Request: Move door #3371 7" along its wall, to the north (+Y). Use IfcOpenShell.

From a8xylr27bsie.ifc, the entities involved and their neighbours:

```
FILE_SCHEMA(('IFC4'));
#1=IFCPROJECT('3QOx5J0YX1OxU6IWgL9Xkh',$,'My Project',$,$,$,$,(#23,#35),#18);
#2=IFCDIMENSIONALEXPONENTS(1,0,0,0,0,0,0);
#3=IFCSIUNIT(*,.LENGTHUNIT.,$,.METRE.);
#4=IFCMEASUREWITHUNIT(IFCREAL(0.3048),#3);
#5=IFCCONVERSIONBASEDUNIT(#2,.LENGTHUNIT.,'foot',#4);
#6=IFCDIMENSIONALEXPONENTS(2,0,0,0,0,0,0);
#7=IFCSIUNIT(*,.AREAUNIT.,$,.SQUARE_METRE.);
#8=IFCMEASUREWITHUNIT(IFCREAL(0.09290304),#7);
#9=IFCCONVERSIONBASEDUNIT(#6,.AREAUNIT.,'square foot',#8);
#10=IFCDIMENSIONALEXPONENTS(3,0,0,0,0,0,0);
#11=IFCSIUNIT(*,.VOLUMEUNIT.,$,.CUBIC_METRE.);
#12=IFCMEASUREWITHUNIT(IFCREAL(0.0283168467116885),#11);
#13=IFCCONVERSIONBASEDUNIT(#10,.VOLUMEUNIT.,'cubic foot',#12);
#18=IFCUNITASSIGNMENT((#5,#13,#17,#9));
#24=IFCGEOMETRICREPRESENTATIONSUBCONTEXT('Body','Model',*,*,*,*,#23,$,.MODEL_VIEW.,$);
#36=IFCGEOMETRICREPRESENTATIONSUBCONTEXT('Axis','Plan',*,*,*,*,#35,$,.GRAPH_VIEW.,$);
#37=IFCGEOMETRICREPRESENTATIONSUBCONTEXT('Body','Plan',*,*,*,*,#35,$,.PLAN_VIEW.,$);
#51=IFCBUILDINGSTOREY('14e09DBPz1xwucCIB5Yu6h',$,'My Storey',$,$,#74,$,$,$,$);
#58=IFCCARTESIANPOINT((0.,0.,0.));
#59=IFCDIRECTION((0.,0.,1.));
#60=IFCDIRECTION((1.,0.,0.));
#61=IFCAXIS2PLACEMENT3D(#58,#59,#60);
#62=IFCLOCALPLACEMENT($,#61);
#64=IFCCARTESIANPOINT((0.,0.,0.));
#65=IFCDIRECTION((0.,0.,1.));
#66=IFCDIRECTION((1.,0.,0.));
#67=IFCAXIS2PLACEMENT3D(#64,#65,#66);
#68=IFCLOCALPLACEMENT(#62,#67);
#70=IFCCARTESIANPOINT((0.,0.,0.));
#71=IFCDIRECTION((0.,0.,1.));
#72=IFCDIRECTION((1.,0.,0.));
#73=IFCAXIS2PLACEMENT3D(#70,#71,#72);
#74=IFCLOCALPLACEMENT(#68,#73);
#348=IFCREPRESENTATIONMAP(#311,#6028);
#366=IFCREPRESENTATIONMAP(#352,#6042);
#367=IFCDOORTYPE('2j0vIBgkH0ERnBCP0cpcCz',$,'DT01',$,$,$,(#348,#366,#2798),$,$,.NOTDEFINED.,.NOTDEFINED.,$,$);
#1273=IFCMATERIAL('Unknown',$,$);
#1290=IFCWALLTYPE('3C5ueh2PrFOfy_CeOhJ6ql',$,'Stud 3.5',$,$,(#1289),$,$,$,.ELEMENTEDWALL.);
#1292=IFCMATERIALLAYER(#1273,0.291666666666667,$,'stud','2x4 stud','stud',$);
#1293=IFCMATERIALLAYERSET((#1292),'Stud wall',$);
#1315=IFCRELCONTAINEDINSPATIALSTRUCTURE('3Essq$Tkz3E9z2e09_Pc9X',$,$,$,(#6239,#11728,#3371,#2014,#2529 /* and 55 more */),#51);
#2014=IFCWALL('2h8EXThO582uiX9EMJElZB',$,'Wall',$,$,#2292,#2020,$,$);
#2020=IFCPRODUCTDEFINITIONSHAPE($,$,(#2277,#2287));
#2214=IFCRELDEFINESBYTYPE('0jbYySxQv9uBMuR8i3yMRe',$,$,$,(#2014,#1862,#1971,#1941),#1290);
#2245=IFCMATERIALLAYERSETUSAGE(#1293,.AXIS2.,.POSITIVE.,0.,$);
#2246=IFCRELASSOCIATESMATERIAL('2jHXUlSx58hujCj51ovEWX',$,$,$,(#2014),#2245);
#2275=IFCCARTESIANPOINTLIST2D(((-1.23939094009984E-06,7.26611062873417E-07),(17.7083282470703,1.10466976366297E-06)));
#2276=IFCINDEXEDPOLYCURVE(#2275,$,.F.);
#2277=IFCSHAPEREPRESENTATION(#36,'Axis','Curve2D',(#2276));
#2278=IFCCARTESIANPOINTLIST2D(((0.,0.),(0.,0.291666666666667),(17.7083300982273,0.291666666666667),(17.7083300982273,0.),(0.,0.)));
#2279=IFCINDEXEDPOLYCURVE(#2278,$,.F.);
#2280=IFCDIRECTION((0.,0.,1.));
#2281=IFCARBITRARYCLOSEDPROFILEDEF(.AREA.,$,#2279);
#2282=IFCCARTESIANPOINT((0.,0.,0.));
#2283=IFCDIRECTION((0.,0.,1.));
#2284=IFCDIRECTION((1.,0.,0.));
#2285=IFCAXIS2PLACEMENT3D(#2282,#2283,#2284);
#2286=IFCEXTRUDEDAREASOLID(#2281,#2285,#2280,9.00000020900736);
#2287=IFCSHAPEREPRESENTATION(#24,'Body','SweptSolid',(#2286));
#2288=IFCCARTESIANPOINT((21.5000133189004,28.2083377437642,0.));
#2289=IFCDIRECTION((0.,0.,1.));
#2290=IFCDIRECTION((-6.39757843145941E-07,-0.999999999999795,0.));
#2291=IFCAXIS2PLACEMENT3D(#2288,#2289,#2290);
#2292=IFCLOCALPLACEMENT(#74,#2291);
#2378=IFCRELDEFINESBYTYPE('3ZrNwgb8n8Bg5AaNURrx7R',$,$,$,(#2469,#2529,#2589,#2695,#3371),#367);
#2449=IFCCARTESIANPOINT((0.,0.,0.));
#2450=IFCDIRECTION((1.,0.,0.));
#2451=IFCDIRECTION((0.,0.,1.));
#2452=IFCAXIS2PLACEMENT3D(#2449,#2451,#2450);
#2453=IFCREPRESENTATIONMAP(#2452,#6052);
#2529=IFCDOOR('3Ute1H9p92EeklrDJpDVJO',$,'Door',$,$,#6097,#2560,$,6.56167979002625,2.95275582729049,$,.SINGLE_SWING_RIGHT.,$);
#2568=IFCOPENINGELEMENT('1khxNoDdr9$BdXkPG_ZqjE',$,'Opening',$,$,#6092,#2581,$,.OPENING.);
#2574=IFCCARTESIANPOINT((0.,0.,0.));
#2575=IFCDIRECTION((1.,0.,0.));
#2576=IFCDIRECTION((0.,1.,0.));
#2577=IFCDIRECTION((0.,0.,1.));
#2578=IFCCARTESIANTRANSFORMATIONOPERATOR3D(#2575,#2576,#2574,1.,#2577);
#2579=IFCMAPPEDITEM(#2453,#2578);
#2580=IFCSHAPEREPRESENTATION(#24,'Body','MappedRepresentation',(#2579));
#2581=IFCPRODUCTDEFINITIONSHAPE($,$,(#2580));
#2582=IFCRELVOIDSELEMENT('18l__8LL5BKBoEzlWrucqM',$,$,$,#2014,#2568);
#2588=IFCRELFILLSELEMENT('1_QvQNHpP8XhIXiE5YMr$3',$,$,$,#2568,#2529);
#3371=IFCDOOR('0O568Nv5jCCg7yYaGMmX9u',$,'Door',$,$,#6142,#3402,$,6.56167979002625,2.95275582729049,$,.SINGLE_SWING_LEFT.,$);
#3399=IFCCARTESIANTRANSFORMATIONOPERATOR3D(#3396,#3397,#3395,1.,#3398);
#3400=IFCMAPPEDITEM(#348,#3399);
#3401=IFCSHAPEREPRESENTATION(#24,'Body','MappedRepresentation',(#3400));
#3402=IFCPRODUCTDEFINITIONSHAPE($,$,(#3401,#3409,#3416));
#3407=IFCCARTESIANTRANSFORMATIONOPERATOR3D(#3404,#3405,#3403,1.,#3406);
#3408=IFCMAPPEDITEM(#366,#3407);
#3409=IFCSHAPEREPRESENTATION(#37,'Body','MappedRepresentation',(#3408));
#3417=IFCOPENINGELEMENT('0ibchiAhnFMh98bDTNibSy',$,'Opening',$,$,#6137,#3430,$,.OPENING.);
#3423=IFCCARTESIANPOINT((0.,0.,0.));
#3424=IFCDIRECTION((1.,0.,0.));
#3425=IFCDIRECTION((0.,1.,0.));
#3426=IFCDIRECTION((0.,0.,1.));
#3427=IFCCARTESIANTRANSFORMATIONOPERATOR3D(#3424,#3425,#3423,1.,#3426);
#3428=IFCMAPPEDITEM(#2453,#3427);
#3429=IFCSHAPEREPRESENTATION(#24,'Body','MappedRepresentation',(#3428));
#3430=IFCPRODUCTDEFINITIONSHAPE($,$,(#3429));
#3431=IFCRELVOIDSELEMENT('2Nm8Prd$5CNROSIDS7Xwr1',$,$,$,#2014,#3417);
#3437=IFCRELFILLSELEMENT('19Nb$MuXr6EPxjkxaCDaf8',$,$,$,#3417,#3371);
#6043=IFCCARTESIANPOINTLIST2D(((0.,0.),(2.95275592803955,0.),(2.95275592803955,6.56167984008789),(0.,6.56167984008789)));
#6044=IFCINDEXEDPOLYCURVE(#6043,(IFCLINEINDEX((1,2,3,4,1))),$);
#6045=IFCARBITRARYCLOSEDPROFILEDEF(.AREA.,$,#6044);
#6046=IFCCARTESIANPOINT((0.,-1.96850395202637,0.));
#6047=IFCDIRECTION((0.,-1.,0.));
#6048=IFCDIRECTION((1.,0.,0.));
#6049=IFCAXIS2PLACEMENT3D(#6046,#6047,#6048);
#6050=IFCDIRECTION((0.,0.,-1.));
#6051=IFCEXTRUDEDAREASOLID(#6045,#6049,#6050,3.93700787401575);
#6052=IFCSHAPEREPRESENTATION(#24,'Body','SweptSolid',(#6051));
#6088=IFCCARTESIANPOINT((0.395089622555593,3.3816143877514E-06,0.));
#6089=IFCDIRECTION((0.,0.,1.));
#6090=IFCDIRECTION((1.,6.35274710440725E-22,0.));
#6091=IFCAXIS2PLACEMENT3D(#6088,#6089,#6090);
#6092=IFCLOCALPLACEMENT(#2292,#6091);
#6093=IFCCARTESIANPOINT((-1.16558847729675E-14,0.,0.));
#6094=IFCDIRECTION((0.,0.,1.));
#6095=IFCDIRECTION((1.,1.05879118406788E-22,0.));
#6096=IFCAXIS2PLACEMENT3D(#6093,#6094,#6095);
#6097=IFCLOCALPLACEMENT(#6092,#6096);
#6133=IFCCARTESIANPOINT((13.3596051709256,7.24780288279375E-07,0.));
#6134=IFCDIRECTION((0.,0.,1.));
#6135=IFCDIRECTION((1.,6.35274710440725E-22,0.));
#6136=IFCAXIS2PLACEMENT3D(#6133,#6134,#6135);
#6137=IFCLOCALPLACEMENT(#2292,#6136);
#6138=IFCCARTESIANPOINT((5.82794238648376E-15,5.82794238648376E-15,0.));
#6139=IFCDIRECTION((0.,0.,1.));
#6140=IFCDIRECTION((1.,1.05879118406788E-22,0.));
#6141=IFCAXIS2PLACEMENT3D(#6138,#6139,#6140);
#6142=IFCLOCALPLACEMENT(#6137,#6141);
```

```python
import ifcopenshell
import ifcopenshell.api.geometry
import ifcopenshell.util.placement
import ifcopenshell.util.unit

model = ifcopenshell.open("a8xylr27bsie.ifc")
unit_scale = ifcopenshell.util.unit.calculate_unit_scale(model)

door = model.by_guid("0O568Nv5jCCg7yYaGMmX9u")
opening = door.FillsVoids[0].RelatingOpeningElement
wall = opening.VoidsElements[0].RelatingBuildingElement

wall_matrix = ifcopenshell.util.placement.get_local_placement(wall.ObjectPlacement)
shift = wall_matrix[:3, 0] * -7 * 0.0254 / unit_scale
before = ifcopenshell.util.placement.get_local_placement(door.ObjectPlacement)[:3, 3].copy()

# The door is placed relative to its opening, so it follows when the opening moves.
matrix = ifcopenshell.util.placement.get_local_placement(opening.ObjectPlacement)
matrix[:3, 3] += shift
ifcopenshell.api.geometry.edit_object_placement(
    model, product=opening, matrix=matrix, is_si=False, should_transform_children=True
)

after = ifcopenshell.util.placement.get_local_placement(door.ObjectPlacement)[:3, 3]
print("door moved by", (after - before).round(3) + 0.0)

model.write("a8xylr27bsie-out.ifc")
```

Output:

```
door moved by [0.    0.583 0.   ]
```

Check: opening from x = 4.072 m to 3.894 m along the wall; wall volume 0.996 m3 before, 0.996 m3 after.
